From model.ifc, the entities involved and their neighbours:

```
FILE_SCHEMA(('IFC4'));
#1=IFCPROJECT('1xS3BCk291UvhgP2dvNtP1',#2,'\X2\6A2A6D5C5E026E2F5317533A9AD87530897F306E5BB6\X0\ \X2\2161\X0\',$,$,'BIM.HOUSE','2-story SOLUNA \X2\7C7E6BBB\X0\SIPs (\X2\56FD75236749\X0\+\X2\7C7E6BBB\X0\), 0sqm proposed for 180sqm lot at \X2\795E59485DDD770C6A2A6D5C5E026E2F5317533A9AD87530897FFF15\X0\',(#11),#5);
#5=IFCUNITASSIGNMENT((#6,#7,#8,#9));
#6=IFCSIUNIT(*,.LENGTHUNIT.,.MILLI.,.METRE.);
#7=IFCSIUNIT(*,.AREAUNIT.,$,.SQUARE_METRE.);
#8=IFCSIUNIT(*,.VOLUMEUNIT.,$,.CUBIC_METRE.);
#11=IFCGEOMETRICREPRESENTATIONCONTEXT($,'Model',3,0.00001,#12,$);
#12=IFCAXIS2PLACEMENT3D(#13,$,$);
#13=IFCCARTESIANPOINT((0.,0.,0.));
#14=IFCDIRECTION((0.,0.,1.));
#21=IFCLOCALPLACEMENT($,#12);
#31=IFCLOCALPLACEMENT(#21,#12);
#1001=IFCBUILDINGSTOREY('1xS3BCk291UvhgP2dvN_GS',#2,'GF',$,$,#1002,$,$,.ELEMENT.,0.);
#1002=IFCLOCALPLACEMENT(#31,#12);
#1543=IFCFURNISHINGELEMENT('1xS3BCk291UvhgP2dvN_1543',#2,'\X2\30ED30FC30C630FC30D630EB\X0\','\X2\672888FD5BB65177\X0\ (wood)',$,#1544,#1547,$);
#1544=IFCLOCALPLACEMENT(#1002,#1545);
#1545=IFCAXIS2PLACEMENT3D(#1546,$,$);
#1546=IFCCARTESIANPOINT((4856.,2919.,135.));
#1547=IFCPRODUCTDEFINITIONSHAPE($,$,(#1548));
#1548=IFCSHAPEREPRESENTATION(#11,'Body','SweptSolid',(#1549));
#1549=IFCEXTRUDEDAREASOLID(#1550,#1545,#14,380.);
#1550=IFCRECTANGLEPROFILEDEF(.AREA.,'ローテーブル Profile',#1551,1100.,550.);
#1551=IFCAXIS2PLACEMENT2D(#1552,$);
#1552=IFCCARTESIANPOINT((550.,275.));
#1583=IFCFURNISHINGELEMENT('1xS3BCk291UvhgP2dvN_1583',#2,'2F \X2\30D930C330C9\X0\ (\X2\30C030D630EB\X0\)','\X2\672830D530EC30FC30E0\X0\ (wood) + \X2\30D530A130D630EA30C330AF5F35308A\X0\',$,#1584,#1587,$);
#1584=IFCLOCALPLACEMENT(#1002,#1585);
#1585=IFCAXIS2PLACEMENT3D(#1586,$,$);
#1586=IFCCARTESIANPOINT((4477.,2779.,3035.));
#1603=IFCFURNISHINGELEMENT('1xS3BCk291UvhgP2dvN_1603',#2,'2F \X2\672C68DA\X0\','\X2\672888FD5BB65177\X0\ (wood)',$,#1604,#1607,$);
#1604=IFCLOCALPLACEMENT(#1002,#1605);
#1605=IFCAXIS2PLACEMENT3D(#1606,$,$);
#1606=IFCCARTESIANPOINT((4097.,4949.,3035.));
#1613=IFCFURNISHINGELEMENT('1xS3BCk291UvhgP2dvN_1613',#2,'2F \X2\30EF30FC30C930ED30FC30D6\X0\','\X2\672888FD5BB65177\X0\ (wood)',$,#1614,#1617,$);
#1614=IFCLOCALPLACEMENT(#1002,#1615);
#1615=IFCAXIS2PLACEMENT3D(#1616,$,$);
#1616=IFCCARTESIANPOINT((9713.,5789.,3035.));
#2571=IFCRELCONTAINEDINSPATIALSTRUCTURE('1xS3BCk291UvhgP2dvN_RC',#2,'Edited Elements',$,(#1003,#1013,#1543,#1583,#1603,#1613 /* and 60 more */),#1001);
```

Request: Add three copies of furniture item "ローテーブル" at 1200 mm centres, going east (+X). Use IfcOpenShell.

```python
import numpy as np
import ifcopenshell
import ifcopenshell.api.geometry
import ifcopenshell.api.root
import ifcopenshell.util.element
import ifcopenshell.util.placement

model = ifcopenshell.open("model.ifc")


def reuse_history(source, copy):
    """copy_class also copies each property set's owner history, people and application; keep the originals."""
    for rel in copy.IsDefinedBy:
        if rel.is_a("IfcRelDefinesByProperties") and (history := rel.RelatingPropertyDefinition.OwnerHistory):
            rel.RelatingPropertyDefinition.OwnerHistory = source.OwnerHistory
            ifcopenshell.util.element.remove_deep2(model, history)


source = model.by_id(1543)
base = ifcopenshell.util.placement.get_local_placement(source.ObjectPlacement)
step = np.array([1.0, 0.0, 0.0]) * 1200.0

for i in range(1, 4):
    copy = ifcopenshell.api.root.copy_class(model, product=source)
    copy.Representation = ifcopenshell.util.element.copy_deep(
        model, source.Representation, exclude=["IfcGeometricRepresentationContext", "IfcRepresentationMap"]
    )
    reuse_history(source, copy)
    matrix = base.copy()
    matrix[:3, 3] += i * step
    print("added at", matrix[:3, 3].round(3) + 0.0)
    ifcopenshell.api.geometry.edit_object_placement(model, product=copy, matrix=matrix, is_si=False)

model.write("model_edited.ifc")
```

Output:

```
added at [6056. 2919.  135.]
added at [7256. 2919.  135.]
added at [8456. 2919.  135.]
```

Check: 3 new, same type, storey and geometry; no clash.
